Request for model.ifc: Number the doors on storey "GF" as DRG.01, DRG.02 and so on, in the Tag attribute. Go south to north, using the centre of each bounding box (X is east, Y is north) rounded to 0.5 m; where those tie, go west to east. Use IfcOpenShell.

First a look at what the model holds.

```python
import ifcopenshell
import ifcopenshell.util.element
import ifcopenshell.util.placement

model = ifcopenshell.open("model.ifc")
print(model.schema)
storey = next(s for s in model.by_type("IfcBuildingStorey") if s.Name == "GF")
doors = [e for e in ifcopenshell.util.element.get_decomposition(storey) if e.is_a("IfcDoor")]
for e in sorted(doors, key=lambda e: e.id()):
    origin = ifcopenshell.util.placement.get_local_placement(e.ObjectPlacement)[:3, 3]
    print(e.id(), e.Tag, e.Name, origin.round(2) + 0.0, sep=" | ")
```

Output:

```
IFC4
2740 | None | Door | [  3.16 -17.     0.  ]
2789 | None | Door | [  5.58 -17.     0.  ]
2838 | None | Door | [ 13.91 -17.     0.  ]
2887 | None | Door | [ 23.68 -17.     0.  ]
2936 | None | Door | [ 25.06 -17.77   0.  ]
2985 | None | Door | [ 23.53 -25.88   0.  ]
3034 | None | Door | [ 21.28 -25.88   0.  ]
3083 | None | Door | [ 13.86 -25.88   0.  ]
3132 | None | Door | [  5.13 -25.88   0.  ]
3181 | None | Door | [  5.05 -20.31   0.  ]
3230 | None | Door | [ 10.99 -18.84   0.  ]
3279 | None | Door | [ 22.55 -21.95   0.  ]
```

```python
import ifcopenshell
import ifcopenshell.geom
import ifcopenshell.util.element
import ifcopenshell.util.shape

model = ifcopenshell.open("model.ifc")
settings = ifcopenshell.geom.settings()
settings.set("use-world-coords", True)


def centre(element):
    shape = ifcopenshell.geom.create_shape(settings, element)
    return ifcopenshell.util.shape.get_bbox_centroid(shape.geometry)


storey = next(s for s in model.by_type("IfcBuildingStorey") if s.Name == "GF")
doors = [e for e in ifcopenshell.util.element.get_decomposition(storey) if e.is_a("IfcDoor")]

# Insertion points can sit at a corner or the storey origin, so sort by the geometry (in metres).
centres = {e: centre(e) for e in doors}
doors.sort(key=lambda e: (round(centres[e][1] / 0.5), centres[e][0]))

for i, e in enumerate(doors, start=1):
    number = f"DRG.{i:02d}"
    e.Tag = number
    print(e.id(), number)

model.write("model_updated.ifc")
```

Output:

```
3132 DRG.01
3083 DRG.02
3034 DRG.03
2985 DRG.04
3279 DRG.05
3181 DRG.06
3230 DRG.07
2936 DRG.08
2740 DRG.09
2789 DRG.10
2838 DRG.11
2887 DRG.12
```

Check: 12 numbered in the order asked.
